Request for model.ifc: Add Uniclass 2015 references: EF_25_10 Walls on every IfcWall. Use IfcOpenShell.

First a look at what the model holds.

```python
import ifcopenshell

model = ifcopenshell.open("model.ifc")
print(model.schema)
print("classifications:", [c.Name for c in model.by_type("IfcClassification")])
for ifc_class in ("IfcDoor", "IfcRoof", "IfcStair", "IfcWall", "IfcWindow"):
    print(ifc_class, len(model.by_type(ifc_class)))
```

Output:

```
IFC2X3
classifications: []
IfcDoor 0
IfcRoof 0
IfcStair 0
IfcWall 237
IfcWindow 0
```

```python
import ifcopenshell
import ifcopenshell.api.classification

model = ifcopenshell.open("model.ifc")

# IFC2X3 requires Source and Edition and has no link from the project to the system.
system = model.create_entity("IfcClassification", Source="NBS", Edition="2015", Name="Uniclass 2015")

codes = {
    "IfcWall": ("EF_25_10", "Walls"),
}
for ifc_class, (code, name) in codes.items():
    products = model.by_type(ifc_class)
    ifcopenshell.api.classification.add_reference(
        model, products=products, classification=system, identification=code, name=name
    )
    print(code, len(products))

model.write("model_updated.ifc")
```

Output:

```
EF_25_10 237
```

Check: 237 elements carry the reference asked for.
